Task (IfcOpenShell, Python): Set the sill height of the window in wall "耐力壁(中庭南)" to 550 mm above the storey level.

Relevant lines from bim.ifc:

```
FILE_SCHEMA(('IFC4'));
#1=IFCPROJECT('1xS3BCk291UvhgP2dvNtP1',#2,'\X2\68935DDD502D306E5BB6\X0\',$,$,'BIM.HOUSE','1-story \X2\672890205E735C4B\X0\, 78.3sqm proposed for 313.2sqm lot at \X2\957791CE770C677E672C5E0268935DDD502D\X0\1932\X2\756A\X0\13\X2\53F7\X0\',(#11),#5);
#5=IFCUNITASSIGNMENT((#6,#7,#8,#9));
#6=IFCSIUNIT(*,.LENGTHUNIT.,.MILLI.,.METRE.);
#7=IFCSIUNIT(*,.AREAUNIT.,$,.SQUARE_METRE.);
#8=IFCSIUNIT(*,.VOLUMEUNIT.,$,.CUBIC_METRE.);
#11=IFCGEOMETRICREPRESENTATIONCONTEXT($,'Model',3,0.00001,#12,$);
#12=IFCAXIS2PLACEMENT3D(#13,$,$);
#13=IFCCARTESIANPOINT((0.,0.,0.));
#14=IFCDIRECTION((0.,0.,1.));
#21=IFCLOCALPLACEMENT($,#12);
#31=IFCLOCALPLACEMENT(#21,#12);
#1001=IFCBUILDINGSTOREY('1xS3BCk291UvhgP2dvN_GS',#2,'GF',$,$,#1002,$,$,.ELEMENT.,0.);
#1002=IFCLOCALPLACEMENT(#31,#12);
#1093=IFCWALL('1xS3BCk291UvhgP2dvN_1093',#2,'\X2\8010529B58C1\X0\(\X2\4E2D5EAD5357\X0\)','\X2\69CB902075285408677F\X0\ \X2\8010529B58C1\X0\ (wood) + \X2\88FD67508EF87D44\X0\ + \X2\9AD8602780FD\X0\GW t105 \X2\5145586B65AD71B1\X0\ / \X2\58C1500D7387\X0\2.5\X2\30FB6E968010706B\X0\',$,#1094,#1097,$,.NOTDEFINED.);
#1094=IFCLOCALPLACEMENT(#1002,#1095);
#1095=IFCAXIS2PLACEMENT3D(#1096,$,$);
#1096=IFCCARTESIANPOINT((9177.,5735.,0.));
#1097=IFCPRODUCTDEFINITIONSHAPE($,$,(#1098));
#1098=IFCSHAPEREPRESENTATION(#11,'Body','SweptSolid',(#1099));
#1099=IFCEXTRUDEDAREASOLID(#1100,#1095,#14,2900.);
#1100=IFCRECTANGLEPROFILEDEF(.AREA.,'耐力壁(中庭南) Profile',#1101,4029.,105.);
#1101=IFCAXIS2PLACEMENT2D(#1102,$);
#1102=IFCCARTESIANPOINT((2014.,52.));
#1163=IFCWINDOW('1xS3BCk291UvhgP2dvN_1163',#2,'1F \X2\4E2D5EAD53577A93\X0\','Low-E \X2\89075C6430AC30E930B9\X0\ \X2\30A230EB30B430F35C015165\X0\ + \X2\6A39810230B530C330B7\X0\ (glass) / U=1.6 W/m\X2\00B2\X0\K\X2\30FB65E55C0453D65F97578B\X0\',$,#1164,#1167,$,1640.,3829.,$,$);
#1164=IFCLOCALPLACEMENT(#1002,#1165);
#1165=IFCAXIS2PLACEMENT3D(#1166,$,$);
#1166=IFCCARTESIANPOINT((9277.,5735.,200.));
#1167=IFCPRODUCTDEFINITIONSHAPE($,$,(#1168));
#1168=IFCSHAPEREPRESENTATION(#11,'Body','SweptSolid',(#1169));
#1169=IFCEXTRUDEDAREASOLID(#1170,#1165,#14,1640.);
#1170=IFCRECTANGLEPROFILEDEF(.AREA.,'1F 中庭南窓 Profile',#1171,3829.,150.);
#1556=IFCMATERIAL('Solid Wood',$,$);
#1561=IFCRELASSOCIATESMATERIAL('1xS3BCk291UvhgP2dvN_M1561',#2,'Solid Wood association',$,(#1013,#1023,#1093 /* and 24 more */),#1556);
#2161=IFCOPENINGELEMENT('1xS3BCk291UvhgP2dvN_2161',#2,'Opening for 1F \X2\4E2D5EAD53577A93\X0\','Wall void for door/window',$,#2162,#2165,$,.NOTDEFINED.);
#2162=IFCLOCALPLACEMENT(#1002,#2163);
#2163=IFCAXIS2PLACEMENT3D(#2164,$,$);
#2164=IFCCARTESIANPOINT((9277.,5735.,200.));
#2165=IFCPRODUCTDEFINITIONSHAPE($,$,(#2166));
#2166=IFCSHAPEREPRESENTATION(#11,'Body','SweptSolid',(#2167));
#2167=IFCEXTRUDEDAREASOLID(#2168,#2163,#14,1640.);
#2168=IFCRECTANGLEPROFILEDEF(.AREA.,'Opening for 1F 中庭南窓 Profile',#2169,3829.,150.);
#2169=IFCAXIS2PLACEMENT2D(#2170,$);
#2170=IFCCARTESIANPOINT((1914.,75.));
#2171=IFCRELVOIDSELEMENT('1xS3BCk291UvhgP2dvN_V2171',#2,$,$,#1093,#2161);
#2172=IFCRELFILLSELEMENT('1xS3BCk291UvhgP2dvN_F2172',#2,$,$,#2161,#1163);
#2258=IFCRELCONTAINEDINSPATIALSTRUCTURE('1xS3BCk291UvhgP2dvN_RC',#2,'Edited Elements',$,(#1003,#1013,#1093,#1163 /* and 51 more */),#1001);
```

```python
import numpy as np
import ifcopenshell
import ifcopenshell.api.geometry
import ifcopenshell.geom
import ifcopenshell.util.element
import ifcopenshell.util.placement
import ifcopenshell.util.shape
import ifcopenshell.util.unit

model = ifcopenshell.open("bim.ifc")
unit_scale = ifcopenshell.util.unit.calculate_unit_scale(model)

window = model.by_id(1163)
opening = window.FillsVoids[0].RelatingOpeningElement
storey = ifcopenshell.util.element.get_container(window, ifc_class="IfcBuildingStorey")
level = ifcopenshell.util.placement.get_local_placement(storey.ObjectPlacement)[2, 3]

# The opening's origin need not be at the sill, so measure its lowest point.
shape = ifcopenshell.geom.create_shape(ifcopenshell.geom.settings(), opening)
bottom = ifcopenshell.util.shape.get_shape_bottom_elevation(shape, shape.geometry) / unit_scale
dz = level + 0.55 / unit_scale - bottom

shift = np.array([0.0, 0.0, dz])
# The window is not placed relative to its opening, so move both.
for product in (opening, window):
    matrix = ifcopenshell.util.placement.get_local_placement(product.ObjectPlacement)
    matrix[:3, 3] += shift
    ifcopenshell.api.geometry.edit_object_placement(model, product=product, matrix=matrix, is_si=False)

print(f"moved by {dz * unit_scale:+.3f} m")

model.write("bim_rev.ifc")
```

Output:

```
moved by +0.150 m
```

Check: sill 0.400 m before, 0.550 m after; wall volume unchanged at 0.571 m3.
